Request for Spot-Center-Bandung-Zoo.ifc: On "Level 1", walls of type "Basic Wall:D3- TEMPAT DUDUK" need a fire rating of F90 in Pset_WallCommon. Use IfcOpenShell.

First a look at what the model holds.

```python
import ifcopenshell
import ifcopenshell.util.element

model = ifcopenshell.open("Spot-Center-Bandung-Zoo.ifc")
print(model.schema)
storey = next(s for s in model.by_type("IfcBuildingStorey") if s.Name == "Level 1")
walls = [e for e in ifcopenshell.util.element.get_decomposition(storey) if e.is_a("IfcWall")]
seen = {}
for e in walls:
    element_type = ifcopenshell.util.element.get_type(e)
    key = (element_type.Name if element_type != e and element_type else None, ifcopenshell.util.element.get_pset(e, "Pset_WallCommon", "FireRating"))
    seen[key] = seen.get(key, 0) + 1
for (name, value), count in sorted(seen.items(), key=str):
    print(count, "x", name, "|", value)
```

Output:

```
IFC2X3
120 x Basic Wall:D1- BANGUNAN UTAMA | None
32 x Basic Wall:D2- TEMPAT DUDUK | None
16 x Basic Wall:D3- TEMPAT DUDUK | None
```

```python
import ifcopenshell
import ifcopenshell.api.pset
import ifcopenshell.util.element

model = ifcopenshell.open("Spot-Center-Bandung-Zoo.ifc")

storey = next(s for s in model.by_type("IfcBuildingStorey") if s.Name == "Level 1")
walls = [e for e in ifcopenshell.util.element.get_decomposition(storey) if e.is_a("IfcWall")]

count = 0
for e in walls:
    element_type = ifcopenshell.util.element.get_type(e)
    if element_type in (None, e) or element_type.Name != "Basic Wall:D3- TEMPAT DUDUK":
        continue
    # add_pset returns the element's existing set when there is one.
    pset = ifcopenshell.api.pset.add_pset(model, product=e, name="Pset_WallCommon")
    ifcopenshell.api.pset.edit_pset(model, pset=pset, properties={"FireRating": "F90"})
    count += 1

print(count, "walls updated")

model.write("Spot-Center-Bandung-Zoo_v2.ifc")
```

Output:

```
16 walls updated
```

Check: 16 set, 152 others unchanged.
